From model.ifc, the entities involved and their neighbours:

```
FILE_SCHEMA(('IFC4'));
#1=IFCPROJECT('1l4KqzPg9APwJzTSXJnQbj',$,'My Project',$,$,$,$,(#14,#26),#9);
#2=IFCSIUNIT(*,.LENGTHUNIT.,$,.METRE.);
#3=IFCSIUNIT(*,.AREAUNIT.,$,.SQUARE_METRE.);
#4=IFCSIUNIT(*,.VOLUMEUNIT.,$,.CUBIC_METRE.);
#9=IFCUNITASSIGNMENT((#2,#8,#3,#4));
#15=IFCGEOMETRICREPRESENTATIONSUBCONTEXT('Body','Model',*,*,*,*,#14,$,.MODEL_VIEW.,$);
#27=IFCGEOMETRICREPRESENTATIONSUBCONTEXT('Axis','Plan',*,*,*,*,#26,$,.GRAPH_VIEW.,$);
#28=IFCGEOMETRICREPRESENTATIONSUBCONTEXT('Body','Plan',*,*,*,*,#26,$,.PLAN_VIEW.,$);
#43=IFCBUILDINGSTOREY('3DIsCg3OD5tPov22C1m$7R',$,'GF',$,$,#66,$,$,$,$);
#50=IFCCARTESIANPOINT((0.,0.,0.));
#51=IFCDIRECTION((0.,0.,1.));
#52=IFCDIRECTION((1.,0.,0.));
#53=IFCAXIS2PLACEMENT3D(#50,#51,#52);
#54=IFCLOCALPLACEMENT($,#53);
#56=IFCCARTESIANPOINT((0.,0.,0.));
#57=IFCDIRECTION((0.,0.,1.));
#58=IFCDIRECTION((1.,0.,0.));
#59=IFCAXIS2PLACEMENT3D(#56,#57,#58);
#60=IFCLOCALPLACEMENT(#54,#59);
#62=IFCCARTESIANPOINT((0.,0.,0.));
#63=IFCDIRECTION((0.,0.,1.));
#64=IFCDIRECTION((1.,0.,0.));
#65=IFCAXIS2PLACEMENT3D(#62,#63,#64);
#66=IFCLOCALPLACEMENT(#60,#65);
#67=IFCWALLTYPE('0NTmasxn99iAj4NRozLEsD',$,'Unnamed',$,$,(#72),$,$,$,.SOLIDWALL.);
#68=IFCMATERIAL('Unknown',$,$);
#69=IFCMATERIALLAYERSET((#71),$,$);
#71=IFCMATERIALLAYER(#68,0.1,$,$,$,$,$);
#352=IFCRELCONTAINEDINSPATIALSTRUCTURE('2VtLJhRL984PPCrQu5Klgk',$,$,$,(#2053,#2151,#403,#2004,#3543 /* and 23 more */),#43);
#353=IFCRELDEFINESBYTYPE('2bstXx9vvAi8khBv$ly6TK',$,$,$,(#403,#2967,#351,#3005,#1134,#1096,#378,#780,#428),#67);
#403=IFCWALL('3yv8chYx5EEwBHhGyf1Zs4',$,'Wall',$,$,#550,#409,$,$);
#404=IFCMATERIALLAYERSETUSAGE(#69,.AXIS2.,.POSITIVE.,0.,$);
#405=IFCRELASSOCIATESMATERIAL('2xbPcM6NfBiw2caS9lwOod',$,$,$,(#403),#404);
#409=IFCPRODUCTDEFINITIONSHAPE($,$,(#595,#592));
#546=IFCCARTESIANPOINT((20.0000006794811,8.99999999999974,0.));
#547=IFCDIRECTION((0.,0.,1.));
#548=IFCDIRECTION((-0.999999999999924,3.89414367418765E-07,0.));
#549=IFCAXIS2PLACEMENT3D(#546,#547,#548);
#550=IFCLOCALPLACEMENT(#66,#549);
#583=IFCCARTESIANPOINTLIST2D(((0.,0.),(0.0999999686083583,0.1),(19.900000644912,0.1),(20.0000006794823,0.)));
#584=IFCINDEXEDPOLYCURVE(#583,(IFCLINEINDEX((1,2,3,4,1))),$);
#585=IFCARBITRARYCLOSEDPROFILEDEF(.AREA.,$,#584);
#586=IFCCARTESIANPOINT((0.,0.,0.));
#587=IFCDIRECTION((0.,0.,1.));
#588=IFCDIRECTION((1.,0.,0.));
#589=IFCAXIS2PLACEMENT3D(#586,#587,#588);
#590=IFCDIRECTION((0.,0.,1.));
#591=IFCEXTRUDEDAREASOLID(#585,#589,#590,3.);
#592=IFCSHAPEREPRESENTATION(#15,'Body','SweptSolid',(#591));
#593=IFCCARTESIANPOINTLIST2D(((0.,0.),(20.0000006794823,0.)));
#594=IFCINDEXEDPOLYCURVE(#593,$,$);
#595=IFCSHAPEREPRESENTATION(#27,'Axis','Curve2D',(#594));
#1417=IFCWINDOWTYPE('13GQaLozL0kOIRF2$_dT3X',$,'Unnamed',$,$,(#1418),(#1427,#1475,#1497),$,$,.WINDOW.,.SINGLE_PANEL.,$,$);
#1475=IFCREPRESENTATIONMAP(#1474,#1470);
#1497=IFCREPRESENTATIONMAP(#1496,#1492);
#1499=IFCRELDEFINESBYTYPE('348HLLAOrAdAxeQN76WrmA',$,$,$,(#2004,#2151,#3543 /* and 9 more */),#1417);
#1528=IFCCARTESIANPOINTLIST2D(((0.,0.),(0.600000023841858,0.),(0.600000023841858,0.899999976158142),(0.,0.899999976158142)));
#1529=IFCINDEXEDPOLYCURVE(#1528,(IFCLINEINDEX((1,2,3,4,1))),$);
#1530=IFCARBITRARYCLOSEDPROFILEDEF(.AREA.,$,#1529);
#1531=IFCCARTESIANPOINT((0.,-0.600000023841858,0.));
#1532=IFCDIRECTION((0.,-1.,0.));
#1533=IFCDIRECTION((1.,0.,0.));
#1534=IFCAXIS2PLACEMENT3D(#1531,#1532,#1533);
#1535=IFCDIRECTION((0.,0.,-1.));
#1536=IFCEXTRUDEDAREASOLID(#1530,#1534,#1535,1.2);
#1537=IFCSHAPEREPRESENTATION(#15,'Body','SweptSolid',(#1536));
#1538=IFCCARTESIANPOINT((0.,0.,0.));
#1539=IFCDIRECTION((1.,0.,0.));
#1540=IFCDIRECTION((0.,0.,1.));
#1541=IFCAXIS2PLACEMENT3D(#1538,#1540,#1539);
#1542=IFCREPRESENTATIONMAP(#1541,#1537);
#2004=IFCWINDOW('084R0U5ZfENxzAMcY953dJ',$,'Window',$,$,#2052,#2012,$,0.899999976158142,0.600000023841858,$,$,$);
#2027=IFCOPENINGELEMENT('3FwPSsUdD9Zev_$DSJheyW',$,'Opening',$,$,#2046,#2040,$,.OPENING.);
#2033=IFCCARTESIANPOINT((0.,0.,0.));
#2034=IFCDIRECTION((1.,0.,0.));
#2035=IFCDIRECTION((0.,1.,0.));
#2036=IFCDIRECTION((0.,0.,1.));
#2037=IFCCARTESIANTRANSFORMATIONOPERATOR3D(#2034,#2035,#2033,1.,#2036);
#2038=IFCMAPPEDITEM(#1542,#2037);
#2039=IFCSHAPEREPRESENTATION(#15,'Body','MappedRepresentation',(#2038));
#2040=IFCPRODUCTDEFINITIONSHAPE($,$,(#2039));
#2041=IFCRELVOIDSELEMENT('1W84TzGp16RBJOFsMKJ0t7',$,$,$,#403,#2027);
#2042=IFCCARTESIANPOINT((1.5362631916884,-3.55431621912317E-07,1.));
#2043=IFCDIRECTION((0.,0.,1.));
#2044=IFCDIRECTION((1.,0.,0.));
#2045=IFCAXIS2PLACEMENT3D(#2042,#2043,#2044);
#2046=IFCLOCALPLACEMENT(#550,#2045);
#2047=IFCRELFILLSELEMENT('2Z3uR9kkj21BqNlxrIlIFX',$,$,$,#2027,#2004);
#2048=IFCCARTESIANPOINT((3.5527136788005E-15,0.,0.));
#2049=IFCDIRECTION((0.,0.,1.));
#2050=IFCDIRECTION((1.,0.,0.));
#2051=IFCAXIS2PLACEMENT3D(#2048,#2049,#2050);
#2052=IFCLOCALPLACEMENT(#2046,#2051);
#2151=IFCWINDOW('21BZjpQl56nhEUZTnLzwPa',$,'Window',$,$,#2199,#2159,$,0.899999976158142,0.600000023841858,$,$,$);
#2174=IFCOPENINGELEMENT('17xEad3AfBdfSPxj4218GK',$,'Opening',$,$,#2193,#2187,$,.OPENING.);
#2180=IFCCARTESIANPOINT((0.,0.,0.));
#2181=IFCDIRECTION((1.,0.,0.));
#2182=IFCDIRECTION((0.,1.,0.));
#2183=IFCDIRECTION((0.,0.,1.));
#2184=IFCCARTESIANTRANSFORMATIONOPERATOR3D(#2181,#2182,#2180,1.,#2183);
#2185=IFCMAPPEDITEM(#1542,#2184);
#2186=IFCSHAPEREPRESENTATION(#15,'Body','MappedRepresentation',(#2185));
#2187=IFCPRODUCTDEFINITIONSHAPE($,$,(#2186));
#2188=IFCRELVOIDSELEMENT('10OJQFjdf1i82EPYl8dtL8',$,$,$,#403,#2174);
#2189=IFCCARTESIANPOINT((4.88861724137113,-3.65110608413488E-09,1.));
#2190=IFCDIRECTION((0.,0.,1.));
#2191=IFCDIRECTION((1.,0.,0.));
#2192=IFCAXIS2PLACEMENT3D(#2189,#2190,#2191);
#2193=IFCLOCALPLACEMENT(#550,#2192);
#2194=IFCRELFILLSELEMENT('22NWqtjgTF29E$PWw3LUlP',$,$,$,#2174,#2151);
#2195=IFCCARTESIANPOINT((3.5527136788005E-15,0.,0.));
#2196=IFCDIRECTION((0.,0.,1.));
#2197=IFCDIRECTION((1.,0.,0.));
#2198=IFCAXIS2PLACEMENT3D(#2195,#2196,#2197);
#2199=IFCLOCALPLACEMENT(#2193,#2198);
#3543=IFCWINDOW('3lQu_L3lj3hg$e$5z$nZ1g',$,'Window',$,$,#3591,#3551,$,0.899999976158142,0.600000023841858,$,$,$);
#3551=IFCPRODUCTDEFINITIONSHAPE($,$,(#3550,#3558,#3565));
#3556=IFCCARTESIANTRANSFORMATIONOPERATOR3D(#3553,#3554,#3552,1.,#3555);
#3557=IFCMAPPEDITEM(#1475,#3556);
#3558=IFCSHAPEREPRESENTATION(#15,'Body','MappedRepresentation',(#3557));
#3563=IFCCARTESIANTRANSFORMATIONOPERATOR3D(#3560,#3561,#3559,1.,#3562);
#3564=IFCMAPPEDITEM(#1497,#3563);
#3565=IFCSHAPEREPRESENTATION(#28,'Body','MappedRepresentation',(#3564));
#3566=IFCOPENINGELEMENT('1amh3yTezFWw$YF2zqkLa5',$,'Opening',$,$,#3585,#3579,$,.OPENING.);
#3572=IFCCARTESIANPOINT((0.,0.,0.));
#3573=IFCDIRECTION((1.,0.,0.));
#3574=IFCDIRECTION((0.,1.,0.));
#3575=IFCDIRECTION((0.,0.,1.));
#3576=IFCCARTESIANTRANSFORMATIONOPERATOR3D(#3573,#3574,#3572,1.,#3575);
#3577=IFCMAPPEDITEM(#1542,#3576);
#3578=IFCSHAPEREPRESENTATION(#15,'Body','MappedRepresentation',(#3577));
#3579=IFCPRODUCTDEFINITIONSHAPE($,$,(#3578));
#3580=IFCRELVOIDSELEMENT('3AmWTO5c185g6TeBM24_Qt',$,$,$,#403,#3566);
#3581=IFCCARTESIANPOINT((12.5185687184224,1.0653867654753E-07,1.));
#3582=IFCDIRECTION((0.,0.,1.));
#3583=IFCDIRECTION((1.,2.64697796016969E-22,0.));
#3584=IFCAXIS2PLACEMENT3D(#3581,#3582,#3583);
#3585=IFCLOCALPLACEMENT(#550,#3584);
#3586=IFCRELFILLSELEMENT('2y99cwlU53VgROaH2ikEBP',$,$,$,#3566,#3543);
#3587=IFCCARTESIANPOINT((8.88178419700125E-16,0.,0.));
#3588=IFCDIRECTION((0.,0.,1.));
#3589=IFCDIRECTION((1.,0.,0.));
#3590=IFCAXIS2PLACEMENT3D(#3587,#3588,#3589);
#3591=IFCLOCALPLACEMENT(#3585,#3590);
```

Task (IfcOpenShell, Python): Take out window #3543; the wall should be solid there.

```python
import ifcopenshell
import ifcopenshell.api.feature
import ifcopenshell.api.root
import ifcopenshell.geom
import ifcopenshell.util.shape

model = ifcopenshell.open("model.ifc")
settings = ifcopenshell.geom.settings()


def volume(element):
    """Net volume in cubic metres, openings subtracted."""
    shape = ifcopenshell.geom.create_shape(settings, element)
    return ifcopenshell.util.shape.get_volume(shape.geometry)


window = model.by_guid("3lQu_L3lj3hg$e$5z$nZ1g")
opening = window.FillsVoids[0].RelatingOpeningElement
wall = opening.VoidsElements[0].RelatingBuildingElement
before = volume(wall)

ifcopenshell.api.root.remove_product(model, product=window)
ifcopenshell.api.feature.remove_feature(model, feature=opening)

after = volume(wall)

print(f"wall volume {before:.3f} -> {after:.3f} m3")

model.write("model_updated.ifc")
```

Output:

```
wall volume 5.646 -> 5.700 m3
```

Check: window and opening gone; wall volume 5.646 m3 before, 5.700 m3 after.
